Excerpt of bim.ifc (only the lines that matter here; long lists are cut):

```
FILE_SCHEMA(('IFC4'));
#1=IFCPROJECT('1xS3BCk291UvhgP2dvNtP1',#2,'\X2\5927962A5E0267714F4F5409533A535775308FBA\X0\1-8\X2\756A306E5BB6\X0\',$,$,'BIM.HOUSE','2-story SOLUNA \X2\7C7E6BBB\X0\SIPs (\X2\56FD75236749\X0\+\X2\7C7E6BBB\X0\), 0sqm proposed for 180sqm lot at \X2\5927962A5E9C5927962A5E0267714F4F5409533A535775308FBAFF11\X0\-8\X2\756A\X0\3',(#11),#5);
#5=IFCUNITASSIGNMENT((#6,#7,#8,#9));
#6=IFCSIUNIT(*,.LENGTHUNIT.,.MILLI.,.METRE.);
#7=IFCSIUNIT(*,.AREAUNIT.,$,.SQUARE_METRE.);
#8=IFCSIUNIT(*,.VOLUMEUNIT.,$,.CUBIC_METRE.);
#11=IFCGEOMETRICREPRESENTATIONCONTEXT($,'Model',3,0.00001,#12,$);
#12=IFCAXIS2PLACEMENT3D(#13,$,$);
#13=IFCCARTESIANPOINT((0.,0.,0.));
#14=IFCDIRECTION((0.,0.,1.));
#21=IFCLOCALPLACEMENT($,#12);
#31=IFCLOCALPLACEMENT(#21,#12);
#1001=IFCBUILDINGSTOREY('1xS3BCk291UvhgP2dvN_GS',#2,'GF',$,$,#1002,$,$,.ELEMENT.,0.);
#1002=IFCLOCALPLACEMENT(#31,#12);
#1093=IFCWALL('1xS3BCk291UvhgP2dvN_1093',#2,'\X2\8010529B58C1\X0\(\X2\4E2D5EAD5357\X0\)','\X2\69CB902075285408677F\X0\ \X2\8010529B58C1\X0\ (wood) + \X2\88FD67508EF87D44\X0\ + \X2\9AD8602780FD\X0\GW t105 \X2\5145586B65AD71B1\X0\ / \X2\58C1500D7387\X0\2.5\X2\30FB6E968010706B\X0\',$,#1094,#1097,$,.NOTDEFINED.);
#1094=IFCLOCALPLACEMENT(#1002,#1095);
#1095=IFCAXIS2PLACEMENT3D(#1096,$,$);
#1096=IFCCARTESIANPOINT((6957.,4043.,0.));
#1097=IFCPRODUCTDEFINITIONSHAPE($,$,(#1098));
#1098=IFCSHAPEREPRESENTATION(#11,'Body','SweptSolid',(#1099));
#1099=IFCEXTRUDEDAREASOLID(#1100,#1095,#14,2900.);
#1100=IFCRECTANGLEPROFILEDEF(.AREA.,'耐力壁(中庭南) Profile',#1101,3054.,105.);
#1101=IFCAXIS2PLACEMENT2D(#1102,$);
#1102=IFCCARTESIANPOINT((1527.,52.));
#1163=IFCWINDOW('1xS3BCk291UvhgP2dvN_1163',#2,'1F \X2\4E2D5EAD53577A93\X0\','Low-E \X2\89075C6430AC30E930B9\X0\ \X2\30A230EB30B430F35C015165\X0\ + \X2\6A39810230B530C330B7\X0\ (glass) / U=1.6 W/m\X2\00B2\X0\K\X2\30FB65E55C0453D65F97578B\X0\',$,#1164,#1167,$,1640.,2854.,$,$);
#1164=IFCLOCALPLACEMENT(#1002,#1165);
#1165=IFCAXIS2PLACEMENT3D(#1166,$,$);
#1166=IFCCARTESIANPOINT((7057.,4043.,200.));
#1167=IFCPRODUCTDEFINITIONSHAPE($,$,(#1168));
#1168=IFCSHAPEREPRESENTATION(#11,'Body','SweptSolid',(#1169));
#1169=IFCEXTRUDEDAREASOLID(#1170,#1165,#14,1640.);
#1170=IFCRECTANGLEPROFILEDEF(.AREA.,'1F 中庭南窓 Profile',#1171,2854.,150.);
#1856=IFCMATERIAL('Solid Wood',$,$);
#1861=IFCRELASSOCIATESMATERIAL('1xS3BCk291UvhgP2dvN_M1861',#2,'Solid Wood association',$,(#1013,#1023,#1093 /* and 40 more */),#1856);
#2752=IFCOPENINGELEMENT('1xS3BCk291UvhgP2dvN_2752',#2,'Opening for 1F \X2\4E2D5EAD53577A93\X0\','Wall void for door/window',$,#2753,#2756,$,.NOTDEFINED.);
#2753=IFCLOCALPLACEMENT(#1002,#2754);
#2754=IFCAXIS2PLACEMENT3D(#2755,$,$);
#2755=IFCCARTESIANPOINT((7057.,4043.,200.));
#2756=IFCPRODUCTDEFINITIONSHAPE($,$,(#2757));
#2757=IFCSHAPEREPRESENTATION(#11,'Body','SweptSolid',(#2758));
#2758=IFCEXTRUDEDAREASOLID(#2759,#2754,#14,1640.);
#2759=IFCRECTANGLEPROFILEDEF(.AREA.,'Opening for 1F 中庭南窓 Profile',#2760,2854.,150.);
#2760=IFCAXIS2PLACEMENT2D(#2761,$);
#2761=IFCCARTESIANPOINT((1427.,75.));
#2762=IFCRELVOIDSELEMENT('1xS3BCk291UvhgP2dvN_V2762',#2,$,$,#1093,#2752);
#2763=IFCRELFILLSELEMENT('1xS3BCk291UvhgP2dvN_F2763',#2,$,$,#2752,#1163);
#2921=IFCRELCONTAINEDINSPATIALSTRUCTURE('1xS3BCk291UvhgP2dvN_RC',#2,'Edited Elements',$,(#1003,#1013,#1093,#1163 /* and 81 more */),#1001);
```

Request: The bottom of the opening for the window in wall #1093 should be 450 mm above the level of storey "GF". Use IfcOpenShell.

```python
import numpy as np
import ifcopenshell
import ifcopenshell.api.geometry
import ifcopenshell.geom
import ifcopenshell.util.element
import ifcopenshell.util.placement
import ifcopenshell.util.shape
import ifcopenshell.util.unit

model = ifcopenshell.open("bim.ifc")
unit_scale = ifcopenshell.util.unit.calculate_unit_scale(model)

window = model.by_guid("1xS3BCk291UvhgP2dvN_1163")
opening = window.FillsVoids[0].RelatingOpeningElement
storey = ifcopenshell.util.element.get_container(window, ifc_class="IfcBuildingStorey")
level = ifcopenshell.util.placement.get_local_placement(storey.ObjectPlacement)[2, 3]

# The opening's origin need not be at the sill, so measure its lowest point.
shape = ifcopenshell.geom.create_shape(ifcopenshell.geom.settings(), opening)
bottom = ifcopenshell.util.shape.get_shape_bottom_elevation(shape, shape.geometry) / unit_scale
dz = level + 450.0 - bottom

shift = np.array([0.0, 0.0, dz])
# The window is not placed relative to its opening, so move both.
for product in (opening, window):
    matrix = ifcopenshell.util.placement.get_local_placement(product.ObjectPlacement)
    matrix[:3, 3] += shift
    ifcopenshell.api.geometry.edit_object_placement(model, product=product, matrix=matrix, is_si=False)

print(f"moved by {dz * unit_scale:+.3f} m")

model.write("bim-out.ifc")
```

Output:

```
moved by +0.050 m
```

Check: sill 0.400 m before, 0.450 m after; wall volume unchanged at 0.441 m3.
